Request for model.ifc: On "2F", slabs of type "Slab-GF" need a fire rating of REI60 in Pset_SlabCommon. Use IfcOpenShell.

First a look at what the model holds.

```python
import ifcopenshell
import ifcopenshell.util.element

model = ifcopenshell.open("model.ifc")
print(model.schema)
storey = next(s for s in model.by_type("IfcBuildingStorey") if s.Name == "2F")
slabs = [e for e in ifcopenshell.util.element.get_decomposition(storey) if e.is_a("IfcSlab")]
seen = {}
for e in slabs:
    element_type = ifcopenshell.util.element.get_type(e)
    key = (element_type.Name if element_type != e and element_type else None, ifcopenshell.util.element.get_pset(e, "Pset_SlabCommon", "FireRating"))
    seen[key] = seen.get(key, 0) + 1
for (name, value), count in sorted(seen.items(), key=str):
    print(count, "x", name, "|", value)
```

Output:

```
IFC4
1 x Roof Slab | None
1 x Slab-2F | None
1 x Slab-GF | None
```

```python
import ifcopenshell
import ifcopenshell.api.pset
import ifcopenshell.util.element

model = ifcopenshell.open("model.ifc")

storey = next(s for s in model.by_type("IfcBuildingStorey") if s.Name == "2F")
slabs = [e for e in ifcopenshell.util.element.get_decomposition(storey) if e.is_a("IfcSlab")]

count = 0
for e in slabs:
    element_type = ifcopenshell.util.element.get_type(e)
    if element_type in (None, e) or element_type.Name != "Slab-GF":
        continue
    # add_pset returns the element's existing set when there is one.
    pset = ifcopenshell.api.pset.add_pset(model, product=e, name="Pset_SlabCommon")
    ifcopenshell.api.pset.edit_pset(model, pset=pset, properties={"FireRating": "REI60"})
    count += 1

print(count, "slabs updated")

model.write("model_edited.ifc")
```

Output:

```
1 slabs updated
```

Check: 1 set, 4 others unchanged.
